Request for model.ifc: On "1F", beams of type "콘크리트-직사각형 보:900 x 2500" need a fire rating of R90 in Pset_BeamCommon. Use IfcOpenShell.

First a look at what the model holds.

```python
import ifcopenshell
import ifcopenshell.util.element

model = ifcopenshell.open("model.ifc")
print(model.schema)
storey = next(s for s in model.by_type("IfcBuildingStorey") if s.Name == "1F")
beams = [e for e in ifcopenshell.util.element.get_decomposition(storey) if e.is_a("IfcBeam")]
seen = {}
for e in beams:
    element_type = ifcopenshell.util.element.get_type(e)
    key = (element_type.Name if element_type != e and element_type else None, ifcopenshell.util.element.get_pset(e, "Pset_BeamCommon", "FireRating"))
    seen[key] = seen.get(key, 0) + 1
for (name, value), count in sorted(seen.items(), key=str):
    print(count, "x", name, "|", value)
```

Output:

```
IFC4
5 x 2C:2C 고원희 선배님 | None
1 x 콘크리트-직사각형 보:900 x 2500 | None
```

```python
import ifcopenshell
import ifcopenshell.api.pset
import ifcopenshell.util.element

model = ifcopenshell.open("model.ifc")

storey = next(s for s in model.by_type("IfcBuildingStorey") if s.Name == "1F")
beams = [e for e in ifcopenshell.util.element.get_decomposition(storey) if e.is_a("IfcBeam")]

count = 0
for e in beams:
    element_type = ifcopenshell.util.element.get_type(e)
    if element_type in (None, e) or element_type.Name != "콘크리트-직사각형 보:900 x 2500":
        continue
    # add_pset returns the element's existing set when there is one.
    pset = ifcopenshell.api.pset.add_pset(model, product=e, name="Pset_BeamCommon")
    ifcopenshell.api.pset.edit_pset(model, pset=pset, properties={"FireRating": "R90"})
    count += 1

print(count, "beams updated")

model.write("model_edited.ifc")
```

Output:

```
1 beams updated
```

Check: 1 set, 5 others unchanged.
